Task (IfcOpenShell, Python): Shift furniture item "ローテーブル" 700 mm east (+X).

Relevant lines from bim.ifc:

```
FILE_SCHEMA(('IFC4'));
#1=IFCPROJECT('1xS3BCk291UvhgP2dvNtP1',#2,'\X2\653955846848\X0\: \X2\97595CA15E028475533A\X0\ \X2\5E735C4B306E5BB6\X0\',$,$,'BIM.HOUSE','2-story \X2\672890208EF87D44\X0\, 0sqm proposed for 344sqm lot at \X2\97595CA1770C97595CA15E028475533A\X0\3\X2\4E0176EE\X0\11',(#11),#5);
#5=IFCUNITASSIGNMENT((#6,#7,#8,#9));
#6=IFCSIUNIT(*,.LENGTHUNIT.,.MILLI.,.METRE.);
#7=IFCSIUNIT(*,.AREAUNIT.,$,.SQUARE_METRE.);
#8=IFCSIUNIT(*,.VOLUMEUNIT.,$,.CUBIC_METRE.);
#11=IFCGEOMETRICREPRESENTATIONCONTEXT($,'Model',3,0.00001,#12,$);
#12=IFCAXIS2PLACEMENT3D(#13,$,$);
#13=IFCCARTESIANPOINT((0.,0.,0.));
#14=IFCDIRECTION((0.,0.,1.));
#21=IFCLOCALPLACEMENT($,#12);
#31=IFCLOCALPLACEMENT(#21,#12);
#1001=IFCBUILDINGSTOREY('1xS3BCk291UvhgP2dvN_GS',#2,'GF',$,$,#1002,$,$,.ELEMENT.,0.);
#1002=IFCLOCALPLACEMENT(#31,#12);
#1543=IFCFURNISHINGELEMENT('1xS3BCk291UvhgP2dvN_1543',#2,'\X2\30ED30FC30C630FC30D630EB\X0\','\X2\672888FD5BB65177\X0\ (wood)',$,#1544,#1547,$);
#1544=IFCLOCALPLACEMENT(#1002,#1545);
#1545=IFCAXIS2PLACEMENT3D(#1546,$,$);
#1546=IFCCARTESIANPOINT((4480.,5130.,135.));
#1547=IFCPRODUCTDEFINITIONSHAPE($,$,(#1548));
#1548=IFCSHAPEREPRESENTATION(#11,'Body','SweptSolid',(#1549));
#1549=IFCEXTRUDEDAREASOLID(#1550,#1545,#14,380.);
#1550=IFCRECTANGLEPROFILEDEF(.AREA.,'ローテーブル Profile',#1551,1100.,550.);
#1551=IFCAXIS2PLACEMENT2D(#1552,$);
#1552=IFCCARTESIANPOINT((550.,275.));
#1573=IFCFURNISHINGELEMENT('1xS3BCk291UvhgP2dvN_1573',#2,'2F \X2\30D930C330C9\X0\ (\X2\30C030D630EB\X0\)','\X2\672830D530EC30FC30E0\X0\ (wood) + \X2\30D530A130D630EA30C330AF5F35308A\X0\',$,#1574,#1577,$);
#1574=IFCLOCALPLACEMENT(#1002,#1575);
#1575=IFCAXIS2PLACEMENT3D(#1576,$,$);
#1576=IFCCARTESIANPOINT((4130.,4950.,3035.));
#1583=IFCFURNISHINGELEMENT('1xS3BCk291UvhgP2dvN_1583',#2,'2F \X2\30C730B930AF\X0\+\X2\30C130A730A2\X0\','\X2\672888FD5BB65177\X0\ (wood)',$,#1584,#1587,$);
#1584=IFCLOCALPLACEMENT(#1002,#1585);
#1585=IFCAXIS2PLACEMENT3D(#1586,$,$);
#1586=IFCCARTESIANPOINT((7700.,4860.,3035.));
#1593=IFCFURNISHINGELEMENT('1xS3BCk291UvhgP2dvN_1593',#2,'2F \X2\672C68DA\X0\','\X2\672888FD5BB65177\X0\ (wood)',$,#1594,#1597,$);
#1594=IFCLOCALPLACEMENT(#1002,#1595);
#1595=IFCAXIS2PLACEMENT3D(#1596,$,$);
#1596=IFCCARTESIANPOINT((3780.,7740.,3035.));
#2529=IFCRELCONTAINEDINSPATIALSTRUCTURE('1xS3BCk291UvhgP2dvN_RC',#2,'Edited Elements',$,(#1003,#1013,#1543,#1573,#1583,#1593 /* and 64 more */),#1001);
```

```python
import ifcopenshell
import ifcopenshell.api.geometry
import ifcopenshell.util.placement
import ifcopenshell.util.unit

model = ifcopenshell.open("bim.ifc")
unit_scale = ifcopenshell.util.unit.calculate_unit_scale(model)

item = model.by_guid("1xS3BCk291UvhgP2dvN_1543")
matrix = ifcopenshell.util.placement.get_local_placement(item.ObjectPlacement)
matrix[0, 3] += 0.7 / unit_scale
ifcopenshell.api.geometry.edit_object_placement(model, product=item, matrix=matrix, is_si=False)

print(ifcopenshell.util.placement.get_local_placement(item.ObjectPlacement).round(3) + 0.0)

model.write("bim_updated.ifc")
```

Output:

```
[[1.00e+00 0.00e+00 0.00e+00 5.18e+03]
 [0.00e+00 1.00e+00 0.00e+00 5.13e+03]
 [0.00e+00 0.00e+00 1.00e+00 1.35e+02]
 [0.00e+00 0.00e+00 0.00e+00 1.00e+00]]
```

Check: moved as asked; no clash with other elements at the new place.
